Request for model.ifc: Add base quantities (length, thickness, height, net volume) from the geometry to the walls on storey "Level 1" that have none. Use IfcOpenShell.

First a look at what the model holds.

```python
import ifcopenshell
import ifcopenshell.util.element
import ifcopenshell.util.unit

model = ifcopenshell.open("model.ifc")
print(model.schema)
for unit_type in ("LENGTHUNIT", "AREAUNIT", "VOLUMEUNIT"):
    print(unit_type, ifcopenshell.util.unit.calculate_unit_scale(model, unit_type))
storey = next(s for s in model.by_type("IfcBuildingStorey") if s.Name == "Level 1")
walls = [e for e in ifcopenshell.util.element.get_decomposition(storey) if e.is_a("IfcWall")]
for e in sorted(walls, key=lambda e: e.id()):
    print(e.id(), e.is_a(), e.Name, list(ifcopenshell.util.element.get_psets(e, qtos_only=True)), sep=" | ")
```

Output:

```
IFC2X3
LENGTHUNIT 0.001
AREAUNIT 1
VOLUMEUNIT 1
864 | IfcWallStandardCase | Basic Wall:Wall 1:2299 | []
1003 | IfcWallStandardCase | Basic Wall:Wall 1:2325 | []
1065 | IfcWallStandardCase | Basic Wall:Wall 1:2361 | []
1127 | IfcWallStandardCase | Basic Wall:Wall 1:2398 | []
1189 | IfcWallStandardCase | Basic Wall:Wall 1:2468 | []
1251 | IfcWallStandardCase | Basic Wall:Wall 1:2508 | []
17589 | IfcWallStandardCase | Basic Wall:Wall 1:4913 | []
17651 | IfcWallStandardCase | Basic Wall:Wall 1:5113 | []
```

```python
import ifcopenshell
import ifcopenshell.api.pset
import ifcopenshell.geom
import ifcopenshell.util.element
import ifcopenshell.util.shape
import ifcopenshell.util.unit

model = ifcopenshell.open("model.ifc")
unit_scale = ifcopenshell.util.unit.calculate_unit_scale(model)
volume_scale = ifcopenshell.util.unit.calculate_unit_scale(model, "VOLUMEUNIT")
settings = ifcopenshell.geom.settings()

storey = next(s for s in model.by_type("IfcBuildingStorey") if s.Name == "Level 1")
walls = [e for e in ifcopenshell.util.element.get_decomposition(storey) if e.is_a("IfcWall")]

for e in sorted(walls, key=lambda e: e.id()):
    if ifcopenshell.util.element.get_psets(e, qtos_only=True, should_inherit=False):
        continue
    # Geometry comes back in metres, in the element's own axes.
    shape = ifcopenshell.geom.create_shape(settings, e)
    values = {
        "Length": ifcopenshell.util.shape.get_x(shape.geometry) / unit_scale,
        "Width": ifcopenshell.util.shape.get_y(shape.geometry) / unit_scale,
        "Height": ifcopenshell.util.shape.get_z(shape.geometry) / unit_scale,
        "NetVolume": ifcopenshell.util.shape.get_volume(shape.geometry) / volume_scale,
    }
    qto = ifcopenshell.api.pset.add_qto(model, product=e, name="BaseQuantities")
    ifcopenshell.api.pset.edit_qto(model, qto=qto, properties=values)
    print(e.id(), {k: round(v, 3) for k, v in values.items()})

model.write("model-out.ifc")
```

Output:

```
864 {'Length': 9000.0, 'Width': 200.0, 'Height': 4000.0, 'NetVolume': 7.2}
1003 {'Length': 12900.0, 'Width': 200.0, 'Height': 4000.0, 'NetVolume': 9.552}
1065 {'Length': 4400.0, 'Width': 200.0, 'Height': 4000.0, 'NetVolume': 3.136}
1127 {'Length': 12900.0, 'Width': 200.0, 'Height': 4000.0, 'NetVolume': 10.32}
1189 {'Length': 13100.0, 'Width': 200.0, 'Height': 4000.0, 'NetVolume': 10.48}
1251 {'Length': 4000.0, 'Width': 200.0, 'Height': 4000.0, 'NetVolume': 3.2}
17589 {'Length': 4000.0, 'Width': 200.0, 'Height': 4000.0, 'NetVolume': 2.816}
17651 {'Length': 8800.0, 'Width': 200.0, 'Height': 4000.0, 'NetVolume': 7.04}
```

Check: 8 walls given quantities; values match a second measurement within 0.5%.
